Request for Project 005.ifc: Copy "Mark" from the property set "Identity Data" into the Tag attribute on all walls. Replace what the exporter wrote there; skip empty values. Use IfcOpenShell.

First a look at what the model holds.

```python
import ifcopenshell
import ifcopenshell.util.element

model = ifcopenshell.open("Project 005.ifc")
print(model.schema)
walls = model.by_type("IfcWall")
print(len(walls), "walls")
for e in walls[:8]:
    source = ifcopenshell.util.element.get_pset(e, "Identity Data", "Mark")
    target = e.Tag
    print(e.id(), repr(source), repr(target), sep=" | ")
```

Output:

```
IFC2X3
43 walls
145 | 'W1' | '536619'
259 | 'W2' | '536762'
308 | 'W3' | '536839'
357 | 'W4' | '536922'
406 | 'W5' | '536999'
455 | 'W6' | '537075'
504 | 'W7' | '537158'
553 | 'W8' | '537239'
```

```python
import ifcopenshell
import ifcopenshell.util.element

model = ifcopenshell.open("Project 005.ifc")

count = 0
for e in model.by_type("IfcWall"):
    value = ifcopenshell.util.element.get_pset(e, "Identity Data", "Mark")
    current = e.Tag
    if not value or not value.strip() or current == value:
        continue
    e.Tag = value
    count += 1

print(count, "walls updated")

model.write("Project 005_edited.ifc")
```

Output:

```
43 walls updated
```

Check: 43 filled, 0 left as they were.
